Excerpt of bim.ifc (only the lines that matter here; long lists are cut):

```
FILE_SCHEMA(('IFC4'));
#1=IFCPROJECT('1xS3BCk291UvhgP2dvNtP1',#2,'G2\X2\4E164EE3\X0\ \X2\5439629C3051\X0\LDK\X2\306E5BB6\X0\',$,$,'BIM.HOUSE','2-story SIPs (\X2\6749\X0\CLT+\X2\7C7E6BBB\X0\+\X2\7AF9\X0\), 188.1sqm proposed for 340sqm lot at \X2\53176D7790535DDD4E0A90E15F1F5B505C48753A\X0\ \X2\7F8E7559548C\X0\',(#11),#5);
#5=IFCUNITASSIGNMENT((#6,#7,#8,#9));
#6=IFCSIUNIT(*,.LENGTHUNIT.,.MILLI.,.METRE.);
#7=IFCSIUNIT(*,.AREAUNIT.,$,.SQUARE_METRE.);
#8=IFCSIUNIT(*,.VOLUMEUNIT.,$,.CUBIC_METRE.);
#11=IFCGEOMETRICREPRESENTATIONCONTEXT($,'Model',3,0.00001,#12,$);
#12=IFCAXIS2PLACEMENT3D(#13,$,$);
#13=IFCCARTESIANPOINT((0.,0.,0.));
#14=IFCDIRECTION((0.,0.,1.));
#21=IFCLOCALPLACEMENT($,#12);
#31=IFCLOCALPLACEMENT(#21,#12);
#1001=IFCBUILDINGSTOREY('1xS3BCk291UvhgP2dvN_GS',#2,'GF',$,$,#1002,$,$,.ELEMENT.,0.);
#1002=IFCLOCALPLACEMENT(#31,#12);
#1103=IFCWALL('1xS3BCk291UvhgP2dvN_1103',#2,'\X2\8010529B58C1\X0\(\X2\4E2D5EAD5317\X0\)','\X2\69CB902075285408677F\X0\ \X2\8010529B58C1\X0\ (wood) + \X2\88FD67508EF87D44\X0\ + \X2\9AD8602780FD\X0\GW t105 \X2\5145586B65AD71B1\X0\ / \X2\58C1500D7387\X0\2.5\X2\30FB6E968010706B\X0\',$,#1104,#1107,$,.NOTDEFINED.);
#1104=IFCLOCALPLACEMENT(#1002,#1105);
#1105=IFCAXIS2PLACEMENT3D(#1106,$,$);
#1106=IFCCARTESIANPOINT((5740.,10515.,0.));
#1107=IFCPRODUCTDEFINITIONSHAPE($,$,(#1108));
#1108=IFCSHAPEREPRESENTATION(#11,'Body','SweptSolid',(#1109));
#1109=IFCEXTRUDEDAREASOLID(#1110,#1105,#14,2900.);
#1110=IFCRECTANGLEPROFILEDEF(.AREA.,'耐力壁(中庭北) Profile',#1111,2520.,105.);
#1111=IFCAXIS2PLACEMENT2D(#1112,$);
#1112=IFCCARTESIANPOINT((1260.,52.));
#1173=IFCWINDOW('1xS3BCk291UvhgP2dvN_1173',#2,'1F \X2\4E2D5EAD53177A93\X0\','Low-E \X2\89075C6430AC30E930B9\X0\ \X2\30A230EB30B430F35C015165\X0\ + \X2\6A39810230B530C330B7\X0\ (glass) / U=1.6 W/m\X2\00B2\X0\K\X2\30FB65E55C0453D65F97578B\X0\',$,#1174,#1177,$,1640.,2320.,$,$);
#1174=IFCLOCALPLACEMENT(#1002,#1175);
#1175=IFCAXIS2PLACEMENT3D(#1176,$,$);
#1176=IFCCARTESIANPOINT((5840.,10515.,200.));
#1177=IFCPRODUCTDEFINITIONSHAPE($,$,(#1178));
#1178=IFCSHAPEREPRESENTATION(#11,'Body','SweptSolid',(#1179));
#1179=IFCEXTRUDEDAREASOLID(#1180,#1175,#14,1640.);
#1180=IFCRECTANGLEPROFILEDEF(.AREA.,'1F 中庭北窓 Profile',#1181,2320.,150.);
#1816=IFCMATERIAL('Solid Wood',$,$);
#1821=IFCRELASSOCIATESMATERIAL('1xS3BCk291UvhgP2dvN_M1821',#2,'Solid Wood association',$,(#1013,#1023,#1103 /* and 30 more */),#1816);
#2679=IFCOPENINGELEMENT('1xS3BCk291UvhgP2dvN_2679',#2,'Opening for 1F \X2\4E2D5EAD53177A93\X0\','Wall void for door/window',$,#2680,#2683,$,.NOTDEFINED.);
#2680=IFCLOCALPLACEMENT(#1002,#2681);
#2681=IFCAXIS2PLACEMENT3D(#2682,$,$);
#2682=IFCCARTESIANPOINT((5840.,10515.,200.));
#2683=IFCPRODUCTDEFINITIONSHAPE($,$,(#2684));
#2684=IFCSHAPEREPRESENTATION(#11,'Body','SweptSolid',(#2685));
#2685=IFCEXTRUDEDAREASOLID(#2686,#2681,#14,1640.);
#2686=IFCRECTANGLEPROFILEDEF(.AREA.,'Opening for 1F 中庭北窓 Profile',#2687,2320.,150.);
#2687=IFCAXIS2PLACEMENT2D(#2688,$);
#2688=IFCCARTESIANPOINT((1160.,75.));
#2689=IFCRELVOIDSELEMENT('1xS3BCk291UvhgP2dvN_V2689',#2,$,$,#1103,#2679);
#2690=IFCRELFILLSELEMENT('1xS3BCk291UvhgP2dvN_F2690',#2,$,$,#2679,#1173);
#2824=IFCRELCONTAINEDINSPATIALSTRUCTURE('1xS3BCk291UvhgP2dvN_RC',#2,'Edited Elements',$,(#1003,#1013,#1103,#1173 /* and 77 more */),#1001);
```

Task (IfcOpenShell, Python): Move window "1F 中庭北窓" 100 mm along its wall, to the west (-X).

```python
import ifcopenshell
import ifcopenshell.api.geometry
import ifcopenshell.util.placement

model = ifcopenshell.open("bim.ifc")

window = model.by_id(1173)
opening = window.FillsVoids[0].RelatingOpeningElement
wall = opening.VoidsElements[0].RelatingBuildingElement

wall_matrix = ifcopenshell.util.placement.get_local_placement(wall.ObjectPlacement)
shift = wall_matrix[:3, 0] * -100.0
before = ifcopenshell.util.placement.get_local_placement(window.ObjectPlacement)[:3, 3].copy()

# The window is not placed relative to its opening, so move both.
for product in (opening, window):
    matrix = ifcopenshell.util.placement.get_local_placement(product.ObjectPlacement)
    matrix[:3, 3] += shift
    ifcopenshell.api.geometry.edit_object_placement(model, product=product, matrix=matrix, is_si=False)

after = ifcopenshell.util.placement.get_local_placement(window.ObjectPlacement)[:3, 3]
print("window moved by", (after - before).round(3) + 0.0)

model.write("bim_v2.ifc")
```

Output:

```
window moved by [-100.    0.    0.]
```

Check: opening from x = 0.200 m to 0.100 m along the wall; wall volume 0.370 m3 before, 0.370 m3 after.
